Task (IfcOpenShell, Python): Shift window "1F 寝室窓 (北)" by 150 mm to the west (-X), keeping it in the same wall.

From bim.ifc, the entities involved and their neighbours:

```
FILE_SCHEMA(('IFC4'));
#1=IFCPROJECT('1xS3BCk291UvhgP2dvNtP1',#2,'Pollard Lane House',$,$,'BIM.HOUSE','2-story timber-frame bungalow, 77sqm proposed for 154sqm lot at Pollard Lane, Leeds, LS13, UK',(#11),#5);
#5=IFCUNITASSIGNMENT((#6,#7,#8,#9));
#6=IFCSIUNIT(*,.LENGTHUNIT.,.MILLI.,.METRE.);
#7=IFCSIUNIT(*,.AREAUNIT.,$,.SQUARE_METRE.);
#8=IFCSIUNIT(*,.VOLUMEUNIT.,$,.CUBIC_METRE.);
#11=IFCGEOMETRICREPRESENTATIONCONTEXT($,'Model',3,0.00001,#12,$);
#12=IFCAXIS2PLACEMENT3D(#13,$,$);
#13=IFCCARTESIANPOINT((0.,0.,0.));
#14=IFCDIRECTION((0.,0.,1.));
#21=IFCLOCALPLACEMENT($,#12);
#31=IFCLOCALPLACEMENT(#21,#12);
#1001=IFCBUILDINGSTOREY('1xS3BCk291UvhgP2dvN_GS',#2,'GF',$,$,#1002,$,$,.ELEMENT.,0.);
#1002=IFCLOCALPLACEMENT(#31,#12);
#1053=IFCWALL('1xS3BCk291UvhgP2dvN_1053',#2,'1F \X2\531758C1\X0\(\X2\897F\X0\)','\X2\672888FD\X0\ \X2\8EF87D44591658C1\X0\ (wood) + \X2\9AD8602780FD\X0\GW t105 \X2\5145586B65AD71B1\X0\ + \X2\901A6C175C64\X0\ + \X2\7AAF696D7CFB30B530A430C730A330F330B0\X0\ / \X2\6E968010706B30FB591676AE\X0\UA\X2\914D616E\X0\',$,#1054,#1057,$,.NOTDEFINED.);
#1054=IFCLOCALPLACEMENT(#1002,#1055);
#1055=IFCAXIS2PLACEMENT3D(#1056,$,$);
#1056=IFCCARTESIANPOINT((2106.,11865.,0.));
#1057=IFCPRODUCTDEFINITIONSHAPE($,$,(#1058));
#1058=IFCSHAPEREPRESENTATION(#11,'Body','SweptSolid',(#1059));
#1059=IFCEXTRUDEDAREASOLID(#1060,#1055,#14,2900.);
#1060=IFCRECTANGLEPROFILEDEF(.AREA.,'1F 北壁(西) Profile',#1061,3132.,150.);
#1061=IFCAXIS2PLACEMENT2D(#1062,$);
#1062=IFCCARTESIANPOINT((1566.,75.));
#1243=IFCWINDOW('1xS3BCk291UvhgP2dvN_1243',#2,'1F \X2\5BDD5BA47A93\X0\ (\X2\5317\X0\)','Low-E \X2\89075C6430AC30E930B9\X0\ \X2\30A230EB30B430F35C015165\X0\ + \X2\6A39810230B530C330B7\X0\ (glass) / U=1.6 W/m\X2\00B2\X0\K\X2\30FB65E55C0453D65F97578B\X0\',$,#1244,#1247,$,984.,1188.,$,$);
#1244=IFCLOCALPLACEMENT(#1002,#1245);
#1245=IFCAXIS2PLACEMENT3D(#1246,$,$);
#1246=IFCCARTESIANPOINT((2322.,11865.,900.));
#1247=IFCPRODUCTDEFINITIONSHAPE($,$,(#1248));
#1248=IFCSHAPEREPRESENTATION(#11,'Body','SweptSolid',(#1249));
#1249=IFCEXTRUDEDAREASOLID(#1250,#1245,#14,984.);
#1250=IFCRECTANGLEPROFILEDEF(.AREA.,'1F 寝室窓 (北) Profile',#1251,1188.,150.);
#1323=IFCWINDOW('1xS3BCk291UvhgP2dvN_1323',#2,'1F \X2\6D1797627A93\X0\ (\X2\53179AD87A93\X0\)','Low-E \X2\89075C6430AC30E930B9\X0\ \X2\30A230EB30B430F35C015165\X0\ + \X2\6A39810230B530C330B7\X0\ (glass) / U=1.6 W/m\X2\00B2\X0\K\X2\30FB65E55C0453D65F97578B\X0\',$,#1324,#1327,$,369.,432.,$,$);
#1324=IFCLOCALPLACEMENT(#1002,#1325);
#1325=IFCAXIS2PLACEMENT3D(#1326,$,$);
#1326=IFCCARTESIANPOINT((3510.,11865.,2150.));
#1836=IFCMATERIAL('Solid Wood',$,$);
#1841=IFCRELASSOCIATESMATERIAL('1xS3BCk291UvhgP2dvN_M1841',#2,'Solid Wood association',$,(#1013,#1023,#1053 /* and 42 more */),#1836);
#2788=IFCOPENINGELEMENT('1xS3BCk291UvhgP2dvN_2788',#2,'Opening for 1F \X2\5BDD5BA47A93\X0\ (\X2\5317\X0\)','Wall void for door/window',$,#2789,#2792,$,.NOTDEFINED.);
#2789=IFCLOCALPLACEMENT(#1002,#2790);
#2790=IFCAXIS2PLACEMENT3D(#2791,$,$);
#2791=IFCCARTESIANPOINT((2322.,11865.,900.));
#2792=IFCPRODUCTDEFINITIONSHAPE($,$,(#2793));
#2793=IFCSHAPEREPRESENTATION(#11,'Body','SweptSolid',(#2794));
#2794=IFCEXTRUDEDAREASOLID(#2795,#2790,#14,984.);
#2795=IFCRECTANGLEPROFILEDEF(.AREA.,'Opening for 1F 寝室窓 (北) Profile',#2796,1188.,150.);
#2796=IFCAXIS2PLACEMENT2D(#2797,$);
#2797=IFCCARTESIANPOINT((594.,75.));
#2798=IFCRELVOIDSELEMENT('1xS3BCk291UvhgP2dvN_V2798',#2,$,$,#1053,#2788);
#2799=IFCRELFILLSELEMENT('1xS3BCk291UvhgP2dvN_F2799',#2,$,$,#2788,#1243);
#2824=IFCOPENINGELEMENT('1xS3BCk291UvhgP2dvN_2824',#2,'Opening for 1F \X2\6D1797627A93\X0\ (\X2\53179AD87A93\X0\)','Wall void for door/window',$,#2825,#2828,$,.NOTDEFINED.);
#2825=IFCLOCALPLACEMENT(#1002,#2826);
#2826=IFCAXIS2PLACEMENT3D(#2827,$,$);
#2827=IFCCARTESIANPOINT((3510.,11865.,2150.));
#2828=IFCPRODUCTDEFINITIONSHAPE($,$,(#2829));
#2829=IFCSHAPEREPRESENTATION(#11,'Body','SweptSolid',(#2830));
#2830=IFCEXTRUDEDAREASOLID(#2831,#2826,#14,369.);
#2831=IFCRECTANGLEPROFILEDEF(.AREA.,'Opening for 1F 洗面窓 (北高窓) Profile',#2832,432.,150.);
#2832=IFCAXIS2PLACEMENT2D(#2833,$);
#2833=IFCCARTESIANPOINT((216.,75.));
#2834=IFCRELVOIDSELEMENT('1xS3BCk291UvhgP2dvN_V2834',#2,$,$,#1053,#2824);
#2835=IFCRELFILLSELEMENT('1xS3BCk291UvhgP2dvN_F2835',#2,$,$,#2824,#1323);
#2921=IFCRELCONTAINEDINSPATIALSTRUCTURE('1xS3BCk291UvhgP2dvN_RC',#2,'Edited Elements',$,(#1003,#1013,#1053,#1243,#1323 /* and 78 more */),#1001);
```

```python
import ifcopenshell
import ifcopenshell.api.geometry
import ifcopenshell.util.placement
import ifcopenshell.util.unit

model = ifcopenshell.open("bim.ifc")
unit_scale = ifcopenshell.util.unit.calculate_unit_scale(model)

window = model.by_guid("1xS3BCk291UvhgP2dvN_1243")
opening = window.FillsVoids[0].RelatingOpeningElement
wall = opening.VoidsElements[0].RelatingBuildingElement

wall_matrix = ifcopenshell.util.placement.get_local_placement(wall.ObjectPlacement)
shift = wall_matrix[:3, 0] * -0.15 / unit_scale
before = ifcopenshell.util.placement.get_local_placement(window.ObjectPlacement)[:3, 3].copy()

# The window is not placed relative to its opening, so move both.
for product in (opening, window):
    matrix = ifcopenshell.util.placement.get_local_placement(product.ObjectPlacement)
    matrix[:3, 3] += shift
    ifcopenshell.api.geometry.edit_object_placement(model, product=product, matrix=matrix, is_si=False)

after = ifcopenshell.util.placement.get_local_placement(window.ObjectPlacement)[:3, 3]
print("window moved by", (after - before).round(3) + 0.0)

model.write("bim_v2.ifc")
```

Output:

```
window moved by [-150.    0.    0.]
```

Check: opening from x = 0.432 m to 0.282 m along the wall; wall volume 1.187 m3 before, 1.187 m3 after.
